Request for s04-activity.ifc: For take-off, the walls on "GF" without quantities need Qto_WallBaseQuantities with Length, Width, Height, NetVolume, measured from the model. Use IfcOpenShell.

First a look at what the model holds.

```python
import ifcopenshell
import ifcopenshell.util.element
import ifcopenshell.util.unit

model = ifcopenshell.open("s04-activity.ifc")
print(model.schema)
for unit_type in ("LENGTHUNIT", "AREAUNIT", "VOLUMEUNIT"):
    print(unit_type, ifcopenshell.util.unit.calculate_unit_scale(model, unit_type))
storey = next(s for s in model.by_type("IfcBuildingStorey") if s.Name == "GF")
walls = [e for e in ifcopenshell.util.element.get_decomposition(storey) if e.is_a("IfcWall")]
for e in sorted(walls, key=lambda e: e.id()):
    print(e.id(), e.is_a(), e.Name, list(ifcopenshell.util.element.get_psets(e, qtos_only=True)), sep=" | ")
```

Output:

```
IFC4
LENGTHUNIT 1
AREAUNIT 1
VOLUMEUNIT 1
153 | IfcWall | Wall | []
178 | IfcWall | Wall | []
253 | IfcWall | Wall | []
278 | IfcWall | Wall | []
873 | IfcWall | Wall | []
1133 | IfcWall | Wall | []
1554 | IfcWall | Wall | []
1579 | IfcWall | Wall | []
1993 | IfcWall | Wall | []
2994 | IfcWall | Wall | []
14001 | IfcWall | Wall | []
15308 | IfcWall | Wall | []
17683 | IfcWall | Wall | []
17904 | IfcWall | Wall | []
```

```python
import ifcopenshell
import ifcopenshell.api.pset
import ifcopenshell.geom
import ifcopenshell.util.element
import ifcopenshell.util.shape
import ifcopenshell.util.unit

model = ifcopenshell.open("s04-activity.ifc")
unit_scale = ifcopenshell.util.unit.calculate_unit_scale(model)
volume_scale = ifcopenshell.util.unit.calculate_unit_scale(model, "VOLUMEUNIT")
settings = ifcopenshell.geom.settings()

storey = next(s for s in model.by_type("IfcBuildingStorey") if s.Name == "GF")
walls = [e for e in ifcopenshell.util.element.get_decomposition(storey) if e.is_a("IfcWall")]

for e in sorted(walls, key=lambda e: e.id()):
    if ifcopenshell.util.element.get_psets(e, qtos_only=True, should_inherit=False):
        continue
    # Geometry comes back in metres, in the element's own axes.
    shape = ifcopenshell.geom.create_shape(settings, e)
    values = {
        "Length": ifcopenshell.util.shape.get_x(shape.geometry) / unit_scale,
        "Width": ifcopenshell.util.shape.get_y(shape.geometry) / unit_scale,
        "Height": ifcopenshell.util.shape.get_z(shape.geometry) / unit_scale,
        "NetVolume": ifcopenshell.util.shape.get_volume(shape.geometry) / volume_scale,
    }
    qto = ifcopenshell.api.pset.add_qto(model, product=e, name="Qto_WallBaseQuantities")
    ifcopenshell.api.pset.edit_qto(model, qto=qto, properties=values)
    print(e.id(), {k: round(v, 3) for k, v in values.items()})

model.write("s04-activity_updated.ifc")
```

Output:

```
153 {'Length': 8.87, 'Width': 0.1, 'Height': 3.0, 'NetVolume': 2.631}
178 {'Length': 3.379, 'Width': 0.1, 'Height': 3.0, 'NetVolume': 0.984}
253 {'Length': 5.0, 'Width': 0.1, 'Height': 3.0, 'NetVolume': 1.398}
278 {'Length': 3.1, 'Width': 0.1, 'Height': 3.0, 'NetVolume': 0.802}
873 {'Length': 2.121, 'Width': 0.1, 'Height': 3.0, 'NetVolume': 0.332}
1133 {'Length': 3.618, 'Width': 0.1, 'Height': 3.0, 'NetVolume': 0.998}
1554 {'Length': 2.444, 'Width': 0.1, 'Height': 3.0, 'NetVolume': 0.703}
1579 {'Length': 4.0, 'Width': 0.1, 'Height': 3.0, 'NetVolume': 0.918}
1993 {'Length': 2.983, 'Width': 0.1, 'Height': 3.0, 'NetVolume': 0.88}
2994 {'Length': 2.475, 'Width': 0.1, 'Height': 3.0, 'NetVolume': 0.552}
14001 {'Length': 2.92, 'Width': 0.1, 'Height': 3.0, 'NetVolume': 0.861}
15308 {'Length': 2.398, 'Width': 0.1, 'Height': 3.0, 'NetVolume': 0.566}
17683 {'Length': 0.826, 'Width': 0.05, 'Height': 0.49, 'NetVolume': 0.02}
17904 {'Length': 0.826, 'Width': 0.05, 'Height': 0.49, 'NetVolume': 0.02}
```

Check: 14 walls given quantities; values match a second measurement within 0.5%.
